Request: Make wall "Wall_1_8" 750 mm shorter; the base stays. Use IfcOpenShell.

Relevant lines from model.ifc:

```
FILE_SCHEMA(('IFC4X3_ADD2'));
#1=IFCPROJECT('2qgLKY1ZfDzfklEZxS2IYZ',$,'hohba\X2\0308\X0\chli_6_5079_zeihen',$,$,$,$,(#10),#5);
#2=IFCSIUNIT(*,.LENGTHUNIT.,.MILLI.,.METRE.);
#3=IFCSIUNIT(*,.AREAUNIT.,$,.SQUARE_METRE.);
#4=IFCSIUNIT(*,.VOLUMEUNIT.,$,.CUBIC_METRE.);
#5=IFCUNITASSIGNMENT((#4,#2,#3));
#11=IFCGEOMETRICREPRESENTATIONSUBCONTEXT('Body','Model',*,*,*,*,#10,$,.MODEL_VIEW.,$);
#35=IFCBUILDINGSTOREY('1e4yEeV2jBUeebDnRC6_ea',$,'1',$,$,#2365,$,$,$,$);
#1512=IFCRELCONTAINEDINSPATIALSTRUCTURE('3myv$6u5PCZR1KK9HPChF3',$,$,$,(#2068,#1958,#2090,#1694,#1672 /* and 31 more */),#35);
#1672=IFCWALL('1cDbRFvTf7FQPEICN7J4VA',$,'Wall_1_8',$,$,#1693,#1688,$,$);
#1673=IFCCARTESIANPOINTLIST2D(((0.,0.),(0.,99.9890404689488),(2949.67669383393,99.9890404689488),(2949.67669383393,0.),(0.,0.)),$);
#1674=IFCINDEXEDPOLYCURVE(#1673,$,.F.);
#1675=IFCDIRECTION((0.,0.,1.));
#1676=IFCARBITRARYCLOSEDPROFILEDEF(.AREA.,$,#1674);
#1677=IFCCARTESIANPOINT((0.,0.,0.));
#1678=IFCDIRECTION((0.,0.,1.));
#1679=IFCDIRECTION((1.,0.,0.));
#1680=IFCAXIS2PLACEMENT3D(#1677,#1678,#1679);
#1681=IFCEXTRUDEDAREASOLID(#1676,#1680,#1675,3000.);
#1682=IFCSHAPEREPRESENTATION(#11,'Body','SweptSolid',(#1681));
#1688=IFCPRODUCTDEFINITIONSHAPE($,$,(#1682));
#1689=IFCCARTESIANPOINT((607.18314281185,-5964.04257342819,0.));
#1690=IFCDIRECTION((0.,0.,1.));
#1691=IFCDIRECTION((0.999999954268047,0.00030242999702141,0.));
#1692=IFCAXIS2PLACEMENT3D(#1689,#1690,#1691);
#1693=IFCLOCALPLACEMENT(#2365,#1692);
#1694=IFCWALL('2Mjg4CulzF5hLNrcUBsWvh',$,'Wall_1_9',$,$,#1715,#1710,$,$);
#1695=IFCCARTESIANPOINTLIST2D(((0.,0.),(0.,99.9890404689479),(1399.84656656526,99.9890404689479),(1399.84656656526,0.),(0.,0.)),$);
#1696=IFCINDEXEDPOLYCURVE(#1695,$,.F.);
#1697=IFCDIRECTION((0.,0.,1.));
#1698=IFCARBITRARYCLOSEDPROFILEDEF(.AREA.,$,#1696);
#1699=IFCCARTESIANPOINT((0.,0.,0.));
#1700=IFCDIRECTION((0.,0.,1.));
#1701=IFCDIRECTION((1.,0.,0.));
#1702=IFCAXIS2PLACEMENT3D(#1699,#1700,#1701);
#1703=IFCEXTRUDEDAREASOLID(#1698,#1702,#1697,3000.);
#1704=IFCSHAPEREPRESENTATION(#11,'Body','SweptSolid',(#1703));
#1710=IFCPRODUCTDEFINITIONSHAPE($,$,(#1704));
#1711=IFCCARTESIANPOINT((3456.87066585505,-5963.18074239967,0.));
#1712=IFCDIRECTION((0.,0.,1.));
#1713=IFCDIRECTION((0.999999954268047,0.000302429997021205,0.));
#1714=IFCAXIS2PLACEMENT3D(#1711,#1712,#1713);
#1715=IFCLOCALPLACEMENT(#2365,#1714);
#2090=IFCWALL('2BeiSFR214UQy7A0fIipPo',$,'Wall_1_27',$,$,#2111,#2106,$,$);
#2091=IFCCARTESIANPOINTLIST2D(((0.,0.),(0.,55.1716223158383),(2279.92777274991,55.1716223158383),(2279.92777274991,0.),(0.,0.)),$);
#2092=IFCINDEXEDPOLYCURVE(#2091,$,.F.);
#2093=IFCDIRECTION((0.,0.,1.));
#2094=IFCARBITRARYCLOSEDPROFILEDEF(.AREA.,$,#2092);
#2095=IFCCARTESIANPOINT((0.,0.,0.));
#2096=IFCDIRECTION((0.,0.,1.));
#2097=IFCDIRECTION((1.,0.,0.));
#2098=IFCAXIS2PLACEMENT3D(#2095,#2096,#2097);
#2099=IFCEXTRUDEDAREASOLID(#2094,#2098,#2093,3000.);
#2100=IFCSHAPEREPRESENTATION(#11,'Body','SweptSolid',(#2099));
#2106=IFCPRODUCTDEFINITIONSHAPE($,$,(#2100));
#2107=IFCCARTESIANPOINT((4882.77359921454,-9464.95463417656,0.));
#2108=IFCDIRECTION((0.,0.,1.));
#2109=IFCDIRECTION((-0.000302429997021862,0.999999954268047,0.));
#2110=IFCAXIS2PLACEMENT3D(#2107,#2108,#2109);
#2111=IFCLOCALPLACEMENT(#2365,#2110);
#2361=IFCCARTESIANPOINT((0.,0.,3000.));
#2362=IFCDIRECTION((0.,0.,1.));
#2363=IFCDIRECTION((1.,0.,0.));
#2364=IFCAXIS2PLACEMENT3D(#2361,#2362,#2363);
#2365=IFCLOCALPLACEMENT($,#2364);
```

```python
import ifcopenshell
import ifcopenshell.geom
import ifcopenshell.util.representation
import ifcopenshell.util.shape
import ifcopenshell.util.unit

model = ifcopenshell.open("model.ifc")
unit_scale = ifcopenshell.util.unit.calculate_unit_scale(model)
settings = ifcopenshell.geom.settings()


def volume(element):
    """Net volume in cubic metres, openings subtracted."""
    shape = ifcopenshell.geom.create_shape(settings, element)
    return ifcopenshell.util.shape.get_volume(shape.geometry)


wall = model.by_id(1672)
before = volume(wall)

body = ifcopenshell.util.representation.get_representation(wall, "Model", "Body")
solid = body.Items[0]
old_height = solid.Depth
solid.Depth -= 0.75 / unit_scale
after = volume(wall)

print(f"height {old_height:g} -> {solid.Depth:g}, volume {before:.3f} -> {after:.3f} m3")

model.write("model-out.ifc")
```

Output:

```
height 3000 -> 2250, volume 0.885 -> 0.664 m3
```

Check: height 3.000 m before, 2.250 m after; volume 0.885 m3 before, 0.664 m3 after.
